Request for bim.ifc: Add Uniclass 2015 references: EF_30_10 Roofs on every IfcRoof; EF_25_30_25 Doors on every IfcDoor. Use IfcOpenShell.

First a look at what the model holds.

```python
import ifcopenshell

model = ifcopenshell.open("bim.ifc")
print(model.schema)
print("classifications:", [c.Name for c in model.by_type("IfcClassification")])
for ifc_class in ("IfcDoor", "IfcRoof", "IfcStair", "IfcWall", "IfcWindow"):
    print(ifc_class, len(model.by_type(ifc_class)))
```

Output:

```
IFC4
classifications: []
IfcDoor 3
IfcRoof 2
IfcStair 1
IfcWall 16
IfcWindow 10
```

```python
import ifcopenshell
import ifcopenshell.api.classification

model = ifcopenshell.open("bim.ifc")

system = ifcopenshell.api.classification.add_classification(model, classification="Uniclass 2015")

codes = {
    "IfcRoof": ("EF_30_10", "Roofs"),
    "IfcDoor": ("EF_25_30_25", "Doors"),
}
for ifc_class, (code, name) in codes.items():
    products = model.by_type(ifc_class)
    ifcopenshell.api.classification.add_reference(
        model, products=products, classification=system, identification=code, name=name
    )
    print(code, len(products))

model.write("bim_edited.ifc")
```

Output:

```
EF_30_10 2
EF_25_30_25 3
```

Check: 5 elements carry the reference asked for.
